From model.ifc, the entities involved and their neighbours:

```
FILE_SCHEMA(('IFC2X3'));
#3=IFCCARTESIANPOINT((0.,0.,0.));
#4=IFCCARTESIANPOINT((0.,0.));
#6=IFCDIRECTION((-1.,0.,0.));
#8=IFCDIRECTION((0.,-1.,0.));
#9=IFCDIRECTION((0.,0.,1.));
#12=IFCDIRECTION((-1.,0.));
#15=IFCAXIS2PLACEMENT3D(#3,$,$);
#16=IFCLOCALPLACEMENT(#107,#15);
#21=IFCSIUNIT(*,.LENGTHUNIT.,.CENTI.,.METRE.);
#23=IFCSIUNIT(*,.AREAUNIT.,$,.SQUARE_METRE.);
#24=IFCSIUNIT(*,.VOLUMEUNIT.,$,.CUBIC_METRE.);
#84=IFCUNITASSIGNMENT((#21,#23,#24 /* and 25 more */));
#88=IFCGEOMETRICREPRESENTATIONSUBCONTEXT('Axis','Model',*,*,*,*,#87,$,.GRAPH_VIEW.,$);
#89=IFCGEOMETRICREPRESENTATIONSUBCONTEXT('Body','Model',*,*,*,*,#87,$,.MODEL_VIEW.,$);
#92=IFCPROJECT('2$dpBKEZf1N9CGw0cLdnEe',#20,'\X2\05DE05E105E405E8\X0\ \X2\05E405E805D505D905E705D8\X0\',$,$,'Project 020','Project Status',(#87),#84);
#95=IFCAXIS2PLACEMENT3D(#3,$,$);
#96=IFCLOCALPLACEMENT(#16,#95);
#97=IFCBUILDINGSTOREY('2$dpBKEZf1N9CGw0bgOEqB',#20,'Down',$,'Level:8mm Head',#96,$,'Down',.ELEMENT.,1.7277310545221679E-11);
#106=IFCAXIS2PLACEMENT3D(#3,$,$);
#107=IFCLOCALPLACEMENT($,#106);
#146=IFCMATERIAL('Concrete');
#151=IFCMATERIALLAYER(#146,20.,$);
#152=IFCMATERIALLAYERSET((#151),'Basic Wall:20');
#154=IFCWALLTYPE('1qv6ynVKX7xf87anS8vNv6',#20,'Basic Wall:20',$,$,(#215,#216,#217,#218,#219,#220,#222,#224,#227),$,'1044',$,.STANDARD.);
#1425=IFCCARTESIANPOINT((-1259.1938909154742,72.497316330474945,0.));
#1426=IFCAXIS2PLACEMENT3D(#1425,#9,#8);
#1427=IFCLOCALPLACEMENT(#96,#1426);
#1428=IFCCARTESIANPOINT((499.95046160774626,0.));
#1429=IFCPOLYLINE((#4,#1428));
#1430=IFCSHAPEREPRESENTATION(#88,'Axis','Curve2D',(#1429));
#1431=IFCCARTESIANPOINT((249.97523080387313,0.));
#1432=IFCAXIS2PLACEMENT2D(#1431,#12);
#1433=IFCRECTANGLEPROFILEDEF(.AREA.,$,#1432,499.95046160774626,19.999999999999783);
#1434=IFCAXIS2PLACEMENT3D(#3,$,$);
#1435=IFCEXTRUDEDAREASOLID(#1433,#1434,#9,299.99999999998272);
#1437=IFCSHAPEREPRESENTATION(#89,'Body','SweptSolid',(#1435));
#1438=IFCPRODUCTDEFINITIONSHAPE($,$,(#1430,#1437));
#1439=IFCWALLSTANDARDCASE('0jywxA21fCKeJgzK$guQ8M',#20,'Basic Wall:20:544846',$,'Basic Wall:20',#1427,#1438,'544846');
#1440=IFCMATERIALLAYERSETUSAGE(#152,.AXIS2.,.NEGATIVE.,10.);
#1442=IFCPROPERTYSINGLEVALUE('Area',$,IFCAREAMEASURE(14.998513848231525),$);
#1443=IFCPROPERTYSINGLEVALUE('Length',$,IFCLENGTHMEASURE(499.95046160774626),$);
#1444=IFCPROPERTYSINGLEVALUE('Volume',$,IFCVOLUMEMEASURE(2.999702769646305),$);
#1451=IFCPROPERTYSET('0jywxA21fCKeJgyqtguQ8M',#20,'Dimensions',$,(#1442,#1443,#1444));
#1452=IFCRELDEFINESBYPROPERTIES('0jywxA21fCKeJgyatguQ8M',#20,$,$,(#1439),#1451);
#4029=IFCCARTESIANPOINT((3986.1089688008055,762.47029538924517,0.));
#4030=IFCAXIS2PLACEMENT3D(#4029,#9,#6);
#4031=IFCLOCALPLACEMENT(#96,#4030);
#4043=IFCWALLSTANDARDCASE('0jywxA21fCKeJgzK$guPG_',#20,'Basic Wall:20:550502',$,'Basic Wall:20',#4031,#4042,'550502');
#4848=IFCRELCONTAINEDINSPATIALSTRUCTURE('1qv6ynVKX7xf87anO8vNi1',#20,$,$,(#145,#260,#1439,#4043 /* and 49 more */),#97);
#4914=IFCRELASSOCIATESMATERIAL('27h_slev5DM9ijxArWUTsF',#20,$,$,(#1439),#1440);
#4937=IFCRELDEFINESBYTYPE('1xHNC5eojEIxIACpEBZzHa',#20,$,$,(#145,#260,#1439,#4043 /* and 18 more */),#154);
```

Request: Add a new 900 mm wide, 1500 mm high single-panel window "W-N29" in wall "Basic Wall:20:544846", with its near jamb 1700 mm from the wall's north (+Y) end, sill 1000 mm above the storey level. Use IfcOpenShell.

```python
import numpy as np
import ifcopenshell
import ifcopenshell.api.feature
import ifcopenshell.api.geometry
import ifcopenshell.api.pset
import ifcopenshell.api.root
import ifcopenshell.api.spatial
import ifcopenshell.api.type
import ifcopenshell.geom
import ifcopenshell.util.element
import ifcopenshell.util.placement
import ifcopenshell.util.representation
import ifcopenshell.util.shape
import ifcopenshell.util.unit

model = ifcopenshell.open("model.ifc")
unit_scale = ifcopenshell.util.unit.calculate_unit_scale(model)
area_scale = ifcopenshell.util.unit.calculate_unit_scale(model, "AREAUNIT")
volume_scale = ifcopenshell.util.unit.calculate_unit_scale(model, "VOLUMEUNIT")
settings = ifcopenshell.geom.settings()


def volume(element):
    """Net volume in cubic metres, openings subtracted."""
    shape = ifcopenshell.geom.create_shape(settings, element)
    return ifcopenshell.util.shape.get_volume(shape.geometry)


wall = model.by_guid("0jywxA21fCKeJgzK$guQ8M")
storey = ifcopenshell.util.element.get_container(wall, ifc_class="IfcBuildingStorey")
context = ifcopenshell.util.representation.get_context(model, "Model", "Body", "MODEL_VIEW")
before = volume(wall)

width, height, from_end, sill = 0.9, 1.5, 1.7, 1  # metres

# The wall runs along its own X axis, and the end named is its -X end.
wall_shape = ifcopenshell.geom.create_shape(settings, wall)
x, y, z = ifcopenshell.util.shape.get_vertices(wall_shape.geometry).T
start = x.min() + from_end
face, thickness = float(y.min()), float(y.max() - y.min())
wall_matrix = ifcopenshell.util.placement.get_local_placement(wall.ObjectPlacement)
level = ifcopenshell.util.placement.get_local_placement(storey.ObjectPlacement)[2, 3]


def in_wall(x, y):
    """Placement at x, y metres in the wall's axes, at sill height."""
    matrix = wall_matrix.copy()
    matrix[:, 3] = wall_matrix @ np.array([x / unit_scale, y / unit_scale, 0.0, 1.0])
    matrix[2, 3] = level + sill / unit_scale
    return matrix


# Opening: a box that overshoots both wall faces by 50 mm.
opening = ifcopenshell.api.root.create_entity(model, ifc_class="IfcOpeningElement")
box = ifcopenshell.api.geometry.add_wall_representation(
    model, context=context, length=width, height=height, thickness=thickness + 0.1
)
ifcopenshell.api.geometry.assign_representation(model, product=opening, representation=box)
ifcopenshell.api.geometry.edit_object_placement(model, product=opening, matrix=in_wall(start, face - 0.05), is_si=False)
ifcopenshell.api.feature.add_feature(model, feature=opening, element=wall)

window = ifcopenshell.api.root.create_entity(model, ifc_class="IfcWindow", name="W-N29")
window.OverallWidth, window.OverallHeight = width / unit_scale, height / unit_scale
body = ifcopenshell.api.geometry.add_window_representation(
    model,
    context=context,
    overall_width=window.OverallWidth,
    overall_height=window.OverallHeight,
    partition_type="SINGLE_PANEL",
)
ifcopenshell.api.geometry.assign_representation(model, product=window, representation=body)
ifcopenshell.api.spatial.assign_container(model, products=[window], relating_structure=storey)
fills = ifcopenshell.api.feature.add_filling(model, opening=opening, element=window)
fills.OwnerHistory = window.OwnerHistory  # required in IFC2X3

# IFC2X3 keeps the operation on the window style.
style = ifcopenshell.api.root.create_entity(model, ifc_class="IfcWindowStyle", name="W-N29")
style.OperationType, style.ConstructionType = "SINGLE_PANEL", "NOTDEFINED"
style.ParameterTakesPrecedence = style.Sizeable = False
ifcopenshell.api.type.assign_type(model, related_objects=[window], relating_type=style)

# Centre the window in the wall's thickness.
ifcopenshell.api.geometry.edit_object_placement(model, product=window, matrix=in_wall(start, face), is_si=False)
window_shape = ifcopenshell.geom.create_shape(settings, window)
depth = ifcopenshell.util.shape.get_vertices(window_shape.geometry)[:, 1]
offset = face + thickness / 2 - (depth.min() + depth.max()) / 2
ifcopenshell.api.geometry.edit_object_placement(model, product=window, matrix=in_wall(start, offset), is_si=False)

after = volume(wall)

# Update the wall's stored quantities.
pset = model.by_id(ifcopenshell.util.element.get_pset(wall, "Dimensions", should_inherit=False)["id"])
ifcopenshell.api.pset.edit_pset(model, pset=pset, properties={
    "Area": model.create_entity("IfcAreaMeasure", after / thickness / area_scale),
    "Volume": model.create_entity("IfcVolumeMeasure", after / volume_scale),
})

print(f"wall volume {before:.3f} -> {after:.3f} m3")

model.write("model_updated.ifc")
```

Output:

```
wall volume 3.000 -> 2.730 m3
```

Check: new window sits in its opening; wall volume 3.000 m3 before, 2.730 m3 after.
